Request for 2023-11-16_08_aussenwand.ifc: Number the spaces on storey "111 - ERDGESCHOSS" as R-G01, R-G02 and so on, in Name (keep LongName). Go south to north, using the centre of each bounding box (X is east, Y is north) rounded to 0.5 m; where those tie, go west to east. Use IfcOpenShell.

First a look at what the model holds.

```python
import ifcopenshell
import ifcopenshell.util.element
import ifcopenshell.util.placement

model = ifcopenshell.open("2023-11-16_08_aussenwand.ifc")
print(model.schema)
storey = next(s for s in model.by_type("IfcBuildingStorey") if s.Name == "111 - ERDGESCHOSS")
spaces = [e for e in ifcopenshell.util.element.get_decomposition(storey) if e.is_a("IfcSpace")]
for e in sorted(spaces, key=lambda e: e.id()):
    origin = ifcopenshell.util.placement.get_local_placement(e.ObjectPlacement)[:3, 3]
    print(e.id(), e.Name, e.LongName, origin.round(2) + 0.0, sep=" | ")
```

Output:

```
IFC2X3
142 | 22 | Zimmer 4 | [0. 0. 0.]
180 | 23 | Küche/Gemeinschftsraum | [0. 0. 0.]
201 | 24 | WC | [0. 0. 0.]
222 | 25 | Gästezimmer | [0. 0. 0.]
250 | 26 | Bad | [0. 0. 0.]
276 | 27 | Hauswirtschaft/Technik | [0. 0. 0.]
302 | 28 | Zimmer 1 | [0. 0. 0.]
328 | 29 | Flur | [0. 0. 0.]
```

```python
import ifcopenshell
import ifcopenshell.geom
import ifcopenshell.util.element
import ifcopenshell.util.shape

model = ifcopenshell.open("2023-11-16_08_aussenwand.ifc")
settings = ifcopenshell.geom.settings()
settings.set("use-world-coords", True)


def centre(element):
    shape = ifcopenshell.geom.create_shape(settings, element)
    return ifcopenshell.util.shape.get_bbox_centroid(shape.geometry)


storey = next(s for s in model.by_type("IfcBuildingStorey") if s.Name == "111 - ERDGESCHOSS")
spaces = [e for e in ifcopenshell.util.element.get_decomposition(storey) if e.is_a("IfcSpace")]

# Insertion points can sit at a corner or the storey origin, so sort by the geometry (in metres).
centres = {e: centre(e) for e in spaces}
spaces.sort(key=lambda e: (round(centres[e][1] / 0.5), centres[e][0]))

for i, e in enumerate(spaces, start=1):
    number = f"R-G{i:02d}"
    e.Name = number
    print(e.id(), number)

model.write("2023-11-16_08_aussenwand_edited.ifc")
```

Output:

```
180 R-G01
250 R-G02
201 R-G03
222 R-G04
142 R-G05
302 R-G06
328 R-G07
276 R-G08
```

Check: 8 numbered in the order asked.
